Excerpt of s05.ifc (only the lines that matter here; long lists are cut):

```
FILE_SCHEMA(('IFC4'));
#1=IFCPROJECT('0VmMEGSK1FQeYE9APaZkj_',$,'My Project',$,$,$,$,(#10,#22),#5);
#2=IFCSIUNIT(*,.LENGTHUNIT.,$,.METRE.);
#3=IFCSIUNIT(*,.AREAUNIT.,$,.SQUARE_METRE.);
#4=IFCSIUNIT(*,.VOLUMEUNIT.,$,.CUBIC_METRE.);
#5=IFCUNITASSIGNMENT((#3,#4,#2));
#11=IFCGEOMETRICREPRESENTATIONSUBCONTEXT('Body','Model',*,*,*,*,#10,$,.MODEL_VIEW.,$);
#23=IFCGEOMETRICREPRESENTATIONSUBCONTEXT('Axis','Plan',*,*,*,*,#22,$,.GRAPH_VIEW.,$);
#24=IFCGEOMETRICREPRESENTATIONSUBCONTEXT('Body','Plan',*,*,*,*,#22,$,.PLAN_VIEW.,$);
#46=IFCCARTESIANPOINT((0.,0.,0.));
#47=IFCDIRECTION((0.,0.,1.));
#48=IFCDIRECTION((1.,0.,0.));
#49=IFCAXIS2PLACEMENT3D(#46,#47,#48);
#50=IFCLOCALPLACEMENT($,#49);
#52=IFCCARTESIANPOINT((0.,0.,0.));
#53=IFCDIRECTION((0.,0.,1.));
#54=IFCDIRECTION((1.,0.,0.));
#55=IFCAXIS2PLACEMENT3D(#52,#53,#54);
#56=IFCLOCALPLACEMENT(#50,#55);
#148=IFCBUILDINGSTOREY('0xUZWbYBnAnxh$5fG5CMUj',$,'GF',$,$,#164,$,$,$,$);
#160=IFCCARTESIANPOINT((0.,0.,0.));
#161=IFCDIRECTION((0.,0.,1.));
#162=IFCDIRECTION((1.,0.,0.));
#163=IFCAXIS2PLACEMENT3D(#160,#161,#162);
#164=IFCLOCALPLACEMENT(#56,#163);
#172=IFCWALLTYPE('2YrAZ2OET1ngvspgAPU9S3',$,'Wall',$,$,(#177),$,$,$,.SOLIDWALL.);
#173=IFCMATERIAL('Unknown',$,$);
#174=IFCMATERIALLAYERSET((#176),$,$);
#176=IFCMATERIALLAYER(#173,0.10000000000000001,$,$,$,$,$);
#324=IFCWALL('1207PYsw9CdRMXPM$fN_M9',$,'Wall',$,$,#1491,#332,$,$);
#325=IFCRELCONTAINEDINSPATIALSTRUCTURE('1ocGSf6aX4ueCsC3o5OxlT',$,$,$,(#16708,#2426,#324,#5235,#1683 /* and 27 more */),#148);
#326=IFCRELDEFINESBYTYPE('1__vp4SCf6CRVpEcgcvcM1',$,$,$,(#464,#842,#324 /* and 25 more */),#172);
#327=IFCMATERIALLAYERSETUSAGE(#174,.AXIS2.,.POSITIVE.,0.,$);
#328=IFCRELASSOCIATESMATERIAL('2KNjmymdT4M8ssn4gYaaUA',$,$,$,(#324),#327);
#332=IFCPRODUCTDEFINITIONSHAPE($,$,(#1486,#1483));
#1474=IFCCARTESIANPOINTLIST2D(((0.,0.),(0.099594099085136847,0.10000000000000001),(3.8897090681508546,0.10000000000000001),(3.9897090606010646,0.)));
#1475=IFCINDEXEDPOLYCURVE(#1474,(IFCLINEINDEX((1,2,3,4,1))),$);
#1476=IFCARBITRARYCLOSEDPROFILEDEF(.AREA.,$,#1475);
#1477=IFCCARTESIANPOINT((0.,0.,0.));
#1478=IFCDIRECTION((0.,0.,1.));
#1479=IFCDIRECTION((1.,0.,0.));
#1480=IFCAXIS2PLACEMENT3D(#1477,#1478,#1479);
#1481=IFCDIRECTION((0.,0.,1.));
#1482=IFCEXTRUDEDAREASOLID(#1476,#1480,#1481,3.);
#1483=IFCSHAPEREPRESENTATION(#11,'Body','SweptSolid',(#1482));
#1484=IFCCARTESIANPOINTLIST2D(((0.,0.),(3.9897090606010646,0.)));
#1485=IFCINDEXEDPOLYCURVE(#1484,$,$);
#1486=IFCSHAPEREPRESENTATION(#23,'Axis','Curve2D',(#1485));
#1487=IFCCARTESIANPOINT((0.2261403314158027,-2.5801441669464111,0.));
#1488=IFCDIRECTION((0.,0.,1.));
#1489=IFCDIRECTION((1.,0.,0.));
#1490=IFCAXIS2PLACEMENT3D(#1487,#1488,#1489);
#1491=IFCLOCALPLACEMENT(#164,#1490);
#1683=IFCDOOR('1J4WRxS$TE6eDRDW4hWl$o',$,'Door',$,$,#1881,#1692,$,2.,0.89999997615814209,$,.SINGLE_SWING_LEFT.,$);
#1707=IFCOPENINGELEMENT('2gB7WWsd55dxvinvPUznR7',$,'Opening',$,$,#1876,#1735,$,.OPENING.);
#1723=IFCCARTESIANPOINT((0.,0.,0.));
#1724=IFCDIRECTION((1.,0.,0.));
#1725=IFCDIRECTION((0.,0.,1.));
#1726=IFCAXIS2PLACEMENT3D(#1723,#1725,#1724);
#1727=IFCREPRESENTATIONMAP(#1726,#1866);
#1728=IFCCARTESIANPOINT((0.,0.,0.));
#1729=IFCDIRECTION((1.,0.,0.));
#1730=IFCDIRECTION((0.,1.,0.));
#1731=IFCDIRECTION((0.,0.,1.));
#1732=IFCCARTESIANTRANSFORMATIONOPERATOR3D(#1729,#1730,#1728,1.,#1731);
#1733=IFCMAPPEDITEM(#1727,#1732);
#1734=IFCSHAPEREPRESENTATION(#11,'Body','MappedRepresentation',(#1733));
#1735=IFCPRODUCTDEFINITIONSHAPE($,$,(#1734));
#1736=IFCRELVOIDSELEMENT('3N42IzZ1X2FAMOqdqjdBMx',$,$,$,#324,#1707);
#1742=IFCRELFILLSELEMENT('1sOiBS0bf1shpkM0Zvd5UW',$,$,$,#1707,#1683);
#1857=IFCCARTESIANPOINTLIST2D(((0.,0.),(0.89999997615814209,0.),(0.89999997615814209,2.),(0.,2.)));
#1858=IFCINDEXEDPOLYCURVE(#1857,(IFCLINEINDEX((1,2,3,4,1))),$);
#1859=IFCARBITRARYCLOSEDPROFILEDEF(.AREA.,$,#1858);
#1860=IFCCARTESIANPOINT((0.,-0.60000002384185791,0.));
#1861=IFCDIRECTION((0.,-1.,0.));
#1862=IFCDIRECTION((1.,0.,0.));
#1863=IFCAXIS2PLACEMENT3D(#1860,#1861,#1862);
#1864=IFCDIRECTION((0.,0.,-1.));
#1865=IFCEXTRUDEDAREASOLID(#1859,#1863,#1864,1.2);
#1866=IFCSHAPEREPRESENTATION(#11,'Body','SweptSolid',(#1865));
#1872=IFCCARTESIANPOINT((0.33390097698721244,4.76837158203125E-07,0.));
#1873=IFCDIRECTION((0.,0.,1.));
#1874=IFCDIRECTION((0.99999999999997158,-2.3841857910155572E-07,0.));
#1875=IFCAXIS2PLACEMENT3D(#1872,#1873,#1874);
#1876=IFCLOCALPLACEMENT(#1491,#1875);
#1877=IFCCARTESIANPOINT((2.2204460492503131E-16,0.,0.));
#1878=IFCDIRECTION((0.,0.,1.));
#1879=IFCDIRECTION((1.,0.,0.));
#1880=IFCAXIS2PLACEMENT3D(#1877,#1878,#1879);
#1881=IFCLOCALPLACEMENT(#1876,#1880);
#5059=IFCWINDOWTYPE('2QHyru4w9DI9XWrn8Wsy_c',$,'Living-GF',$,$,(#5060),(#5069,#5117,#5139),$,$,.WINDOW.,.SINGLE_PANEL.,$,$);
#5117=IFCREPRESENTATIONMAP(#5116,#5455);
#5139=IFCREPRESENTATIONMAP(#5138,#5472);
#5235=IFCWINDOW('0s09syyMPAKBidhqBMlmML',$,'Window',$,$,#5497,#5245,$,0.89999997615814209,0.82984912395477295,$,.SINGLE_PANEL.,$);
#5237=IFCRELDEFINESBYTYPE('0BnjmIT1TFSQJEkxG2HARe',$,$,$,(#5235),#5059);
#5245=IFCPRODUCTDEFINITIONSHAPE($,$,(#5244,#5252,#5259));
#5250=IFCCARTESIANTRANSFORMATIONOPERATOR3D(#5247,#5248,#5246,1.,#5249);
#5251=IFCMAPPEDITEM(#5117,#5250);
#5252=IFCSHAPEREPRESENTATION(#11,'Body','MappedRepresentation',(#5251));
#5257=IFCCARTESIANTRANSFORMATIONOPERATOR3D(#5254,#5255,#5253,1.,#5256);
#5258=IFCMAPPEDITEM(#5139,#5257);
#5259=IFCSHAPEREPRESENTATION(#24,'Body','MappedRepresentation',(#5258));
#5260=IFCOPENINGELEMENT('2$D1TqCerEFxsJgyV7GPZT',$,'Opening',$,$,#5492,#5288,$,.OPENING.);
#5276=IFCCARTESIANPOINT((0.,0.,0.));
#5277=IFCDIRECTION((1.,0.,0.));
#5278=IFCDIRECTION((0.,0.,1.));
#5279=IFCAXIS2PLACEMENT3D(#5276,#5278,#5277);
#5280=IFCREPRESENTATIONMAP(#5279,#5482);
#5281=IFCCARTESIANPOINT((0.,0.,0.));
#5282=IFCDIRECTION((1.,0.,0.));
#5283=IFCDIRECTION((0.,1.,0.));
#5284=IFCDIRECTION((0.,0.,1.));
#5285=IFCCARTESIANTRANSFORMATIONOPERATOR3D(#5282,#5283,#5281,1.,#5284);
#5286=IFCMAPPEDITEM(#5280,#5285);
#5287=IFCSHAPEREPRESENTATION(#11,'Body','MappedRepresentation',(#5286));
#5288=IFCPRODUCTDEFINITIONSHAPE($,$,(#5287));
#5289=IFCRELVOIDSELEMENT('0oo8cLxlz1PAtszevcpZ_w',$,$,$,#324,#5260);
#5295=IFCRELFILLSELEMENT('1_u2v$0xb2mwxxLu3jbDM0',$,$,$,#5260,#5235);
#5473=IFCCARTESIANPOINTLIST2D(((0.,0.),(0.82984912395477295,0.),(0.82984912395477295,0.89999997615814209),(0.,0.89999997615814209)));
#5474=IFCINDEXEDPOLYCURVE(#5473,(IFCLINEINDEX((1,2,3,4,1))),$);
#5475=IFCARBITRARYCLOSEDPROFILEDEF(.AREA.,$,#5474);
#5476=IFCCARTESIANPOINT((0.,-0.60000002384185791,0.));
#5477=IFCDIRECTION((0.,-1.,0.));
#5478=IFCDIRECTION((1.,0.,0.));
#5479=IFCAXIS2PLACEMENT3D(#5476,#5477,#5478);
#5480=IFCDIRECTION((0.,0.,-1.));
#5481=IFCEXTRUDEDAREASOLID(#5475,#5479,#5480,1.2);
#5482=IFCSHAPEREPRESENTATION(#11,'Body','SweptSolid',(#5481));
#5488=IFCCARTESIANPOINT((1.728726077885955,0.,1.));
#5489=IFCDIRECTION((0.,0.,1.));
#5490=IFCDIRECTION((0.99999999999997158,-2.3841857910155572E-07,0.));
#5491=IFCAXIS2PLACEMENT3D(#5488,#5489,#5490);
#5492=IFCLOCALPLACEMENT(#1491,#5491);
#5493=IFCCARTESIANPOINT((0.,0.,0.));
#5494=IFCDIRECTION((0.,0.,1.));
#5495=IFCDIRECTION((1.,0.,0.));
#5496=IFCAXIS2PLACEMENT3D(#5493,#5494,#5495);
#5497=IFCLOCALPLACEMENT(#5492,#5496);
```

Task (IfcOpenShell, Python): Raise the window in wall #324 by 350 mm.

```python
import numpy as np
import ifcopenshell
import ifcopenshell.api.geometry
import ifcopenshell.util.placement
import ifcopenshell.util.unit

model = ifcopenshell.open("s05.ifc")
unit_scale = ifcopenshell.util.unit.calculate_unit_scale(model)

window = model.by_id(5235)
opening = window.FillsVoids[0].RelatingOpeningElement
dz = 0.35 / unit_scale

shift = np.array([0.0, 0.0, dz])
# The window is placed relative to its opening, so it follows when the opening moves.
matrix = ifcopenshell.util.placement.get_local_placement(opening.ObjectPlacement)
matrix[:3, 3] += shift
ifcopenshell.api.geometry.edit_object_placement(
    model, product=opening, matrix=matrix, is_si=False, should_transform_children=True
)

print(f"moved by {dz * unit_scale:+.3f} m")

model.write("s05_updated.ifc")
```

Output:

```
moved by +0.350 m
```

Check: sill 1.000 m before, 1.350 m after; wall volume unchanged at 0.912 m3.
